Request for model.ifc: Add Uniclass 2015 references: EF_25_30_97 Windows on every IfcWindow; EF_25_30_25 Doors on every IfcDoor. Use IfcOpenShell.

First a look at what the model holds.

```python
import ifcopenshell

model = ifcopenshell.open("model.ifc")
print(model.schema)
print("classifications:", [c.Name for c in model.by_type("IfcClassification")])
for ifc_class in ("IfcDoor", "IfcRoof", "IfcStair", "IfcWall", "IfcWindow"):
    print(ifc_class, len(model.by_type(ifc_class)))
```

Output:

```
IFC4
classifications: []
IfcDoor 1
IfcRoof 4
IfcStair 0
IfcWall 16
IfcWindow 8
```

```python
import ifcopenshell
import ifcopenshell.api.classification

model = ifcopenshell.open("model.ifc")

system = ifcopenshell.api.classification.add_classification(model, classification="Uniclass 2015")

codes = {
    "IfcWindow": ("EF_25_30_97", "Windows"),
    "IfcDoor": ("EF_25_30_25", "Doors"),
}
for ifc_class, (code, name) in codes.items():
    products = model.by_type(ifc_class)
    ifcopenshell.api.classification.add_reference(
        model, products=products, classification=system, identification=code, name=name
    )
    print(code, len(products))

model.write("model_updated.ifc")
```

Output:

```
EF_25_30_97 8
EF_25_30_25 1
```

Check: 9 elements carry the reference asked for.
